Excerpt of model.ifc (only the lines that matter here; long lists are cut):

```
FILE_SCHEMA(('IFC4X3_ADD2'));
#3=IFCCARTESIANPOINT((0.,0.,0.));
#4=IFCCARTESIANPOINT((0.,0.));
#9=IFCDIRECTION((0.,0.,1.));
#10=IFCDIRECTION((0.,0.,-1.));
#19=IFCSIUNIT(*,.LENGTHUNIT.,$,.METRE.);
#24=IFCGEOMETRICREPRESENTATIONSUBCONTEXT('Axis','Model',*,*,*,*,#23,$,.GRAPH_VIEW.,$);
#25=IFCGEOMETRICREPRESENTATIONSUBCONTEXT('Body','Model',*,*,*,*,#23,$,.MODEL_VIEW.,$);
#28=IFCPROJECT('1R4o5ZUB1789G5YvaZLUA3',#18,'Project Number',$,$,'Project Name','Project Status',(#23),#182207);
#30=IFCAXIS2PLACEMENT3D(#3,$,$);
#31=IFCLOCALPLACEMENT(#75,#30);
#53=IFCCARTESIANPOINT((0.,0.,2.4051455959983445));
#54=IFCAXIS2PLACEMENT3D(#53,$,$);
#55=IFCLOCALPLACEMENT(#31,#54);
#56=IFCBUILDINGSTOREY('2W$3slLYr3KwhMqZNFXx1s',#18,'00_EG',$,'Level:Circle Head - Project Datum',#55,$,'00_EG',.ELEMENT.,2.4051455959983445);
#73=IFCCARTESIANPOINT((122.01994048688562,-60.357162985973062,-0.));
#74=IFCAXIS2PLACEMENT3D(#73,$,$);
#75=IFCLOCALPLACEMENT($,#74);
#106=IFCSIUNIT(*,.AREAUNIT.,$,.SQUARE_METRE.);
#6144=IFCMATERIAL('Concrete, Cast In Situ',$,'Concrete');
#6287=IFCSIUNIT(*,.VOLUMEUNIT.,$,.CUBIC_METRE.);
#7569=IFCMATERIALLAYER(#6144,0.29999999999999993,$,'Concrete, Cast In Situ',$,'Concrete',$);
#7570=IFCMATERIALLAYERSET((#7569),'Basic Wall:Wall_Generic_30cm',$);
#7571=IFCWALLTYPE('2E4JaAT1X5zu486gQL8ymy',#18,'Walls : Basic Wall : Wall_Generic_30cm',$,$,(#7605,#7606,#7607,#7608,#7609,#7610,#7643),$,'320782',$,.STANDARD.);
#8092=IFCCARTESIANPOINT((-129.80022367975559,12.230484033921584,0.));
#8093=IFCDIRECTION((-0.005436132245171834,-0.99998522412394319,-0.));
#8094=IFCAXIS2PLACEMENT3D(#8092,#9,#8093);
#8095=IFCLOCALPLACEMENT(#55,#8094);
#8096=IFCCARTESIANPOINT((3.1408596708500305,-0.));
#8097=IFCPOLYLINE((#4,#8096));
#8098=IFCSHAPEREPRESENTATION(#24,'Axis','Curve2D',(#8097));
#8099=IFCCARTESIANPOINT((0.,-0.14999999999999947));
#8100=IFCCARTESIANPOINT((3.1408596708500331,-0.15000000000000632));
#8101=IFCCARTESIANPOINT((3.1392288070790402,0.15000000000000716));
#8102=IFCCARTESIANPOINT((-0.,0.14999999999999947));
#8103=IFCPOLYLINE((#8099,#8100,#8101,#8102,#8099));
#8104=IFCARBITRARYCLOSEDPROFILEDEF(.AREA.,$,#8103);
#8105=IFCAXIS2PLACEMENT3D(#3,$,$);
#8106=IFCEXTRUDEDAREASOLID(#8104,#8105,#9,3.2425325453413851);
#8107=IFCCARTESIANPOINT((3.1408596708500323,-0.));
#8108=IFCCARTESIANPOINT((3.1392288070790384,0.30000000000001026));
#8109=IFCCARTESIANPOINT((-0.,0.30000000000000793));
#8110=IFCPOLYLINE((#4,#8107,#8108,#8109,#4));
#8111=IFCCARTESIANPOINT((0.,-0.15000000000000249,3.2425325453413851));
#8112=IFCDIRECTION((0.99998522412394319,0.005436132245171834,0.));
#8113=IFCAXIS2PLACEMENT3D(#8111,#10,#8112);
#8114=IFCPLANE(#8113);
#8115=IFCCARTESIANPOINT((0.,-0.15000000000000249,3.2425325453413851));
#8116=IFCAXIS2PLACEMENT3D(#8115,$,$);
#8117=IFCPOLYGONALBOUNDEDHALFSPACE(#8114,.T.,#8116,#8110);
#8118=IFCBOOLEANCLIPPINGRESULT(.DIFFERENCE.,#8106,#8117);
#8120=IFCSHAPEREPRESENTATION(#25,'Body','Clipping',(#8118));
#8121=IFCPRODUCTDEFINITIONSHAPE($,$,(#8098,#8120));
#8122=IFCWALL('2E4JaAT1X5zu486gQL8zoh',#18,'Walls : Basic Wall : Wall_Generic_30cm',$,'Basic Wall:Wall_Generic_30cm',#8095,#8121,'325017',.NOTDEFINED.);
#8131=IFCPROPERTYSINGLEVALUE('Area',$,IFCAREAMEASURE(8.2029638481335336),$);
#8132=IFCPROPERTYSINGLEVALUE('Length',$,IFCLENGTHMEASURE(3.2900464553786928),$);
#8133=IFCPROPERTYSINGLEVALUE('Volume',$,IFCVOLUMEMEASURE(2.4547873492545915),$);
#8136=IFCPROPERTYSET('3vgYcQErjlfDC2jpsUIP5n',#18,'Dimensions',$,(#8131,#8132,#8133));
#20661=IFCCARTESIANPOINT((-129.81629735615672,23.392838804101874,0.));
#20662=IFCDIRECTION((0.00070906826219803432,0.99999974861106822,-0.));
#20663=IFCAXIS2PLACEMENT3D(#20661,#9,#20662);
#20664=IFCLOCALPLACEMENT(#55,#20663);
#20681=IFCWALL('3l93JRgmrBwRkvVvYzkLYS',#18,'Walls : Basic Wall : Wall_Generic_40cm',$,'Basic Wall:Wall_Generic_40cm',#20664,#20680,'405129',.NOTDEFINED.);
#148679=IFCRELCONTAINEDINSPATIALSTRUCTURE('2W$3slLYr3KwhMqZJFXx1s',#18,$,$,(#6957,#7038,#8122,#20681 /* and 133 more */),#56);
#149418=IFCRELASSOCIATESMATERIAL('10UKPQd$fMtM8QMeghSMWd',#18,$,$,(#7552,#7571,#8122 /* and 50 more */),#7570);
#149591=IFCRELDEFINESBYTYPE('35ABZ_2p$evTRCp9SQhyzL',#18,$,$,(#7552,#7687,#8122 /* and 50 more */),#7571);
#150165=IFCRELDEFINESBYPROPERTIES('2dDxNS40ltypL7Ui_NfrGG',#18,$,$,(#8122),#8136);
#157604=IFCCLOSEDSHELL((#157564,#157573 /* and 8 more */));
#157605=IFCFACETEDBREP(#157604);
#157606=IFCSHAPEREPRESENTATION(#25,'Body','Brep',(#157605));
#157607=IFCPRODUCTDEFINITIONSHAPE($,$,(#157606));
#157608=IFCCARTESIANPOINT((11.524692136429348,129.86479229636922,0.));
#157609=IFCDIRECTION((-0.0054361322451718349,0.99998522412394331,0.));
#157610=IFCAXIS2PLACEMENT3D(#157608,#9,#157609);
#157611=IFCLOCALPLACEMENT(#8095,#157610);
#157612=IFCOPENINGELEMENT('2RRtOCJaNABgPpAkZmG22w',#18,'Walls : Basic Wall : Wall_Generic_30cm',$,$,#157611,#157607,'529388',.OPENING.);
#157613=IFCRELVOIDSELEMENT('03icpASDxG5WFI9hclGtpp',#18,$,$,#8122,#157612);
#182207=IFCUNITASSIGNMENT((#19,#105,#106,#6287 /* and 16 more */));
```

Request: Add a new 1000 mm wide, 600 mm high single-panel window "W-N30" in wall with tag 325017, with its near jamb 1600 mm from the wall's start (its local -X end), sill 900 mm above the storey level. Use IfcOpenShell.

```python
import numpy as np
import ifcopenshell
import ifcopenshell.api.feature
import ifcopenshell.api.geometry
import ifcopenshell.api.pset
import ifcopenshell.api.root
import ifcopenshell.api.spatial
import ifcopenshell.geom
import ifcopenshell.util.element
import ifcopenshell.util.placement
import ifcopenshell.util.representation
import ifcopenshell.util.shape
import ifcopenshell.util.unit

model = ifcopenshell.open("model.ifc")
unit_scale = ifcopenshell.util.unit.calculate_unit_scale(model)
area_scale = ifcopenshell.util.unit.calculate_unit_scale(model, "AREAUNIT")
volume_scale = ifcopenshell.util.unit.calculate_unit_scale(model, "VOLUMEUNIT")
settings = ifcopenshell.geom.settings()


def volume(element):
    """Net volume in cubic metres, openings subtracted."""
    shape = ifcopenshell.geom.create_shape(settings, element)
    return ifcopenshell.util.shape.get_volume(shape.geometry)


wall = model.by_guid("2E4JaAT1X5zu486gQL8zoh")
storey = ifcopenshell.util.element.get_container(wall, ifc_class="IfcBuildingStorey")
context = ifcopenshell.util.representation.get_context(model, "Model", "Body", "MODEL_VIEW")
before = volume(wall)

width, height, from_end, sill = 1, 0.6, 1.6, 0.9  # metres

# The wall runs along its own X axis, and the end named is its -X end.
wall_shape = ifcopenshell.geom.create_shape(settings, wall)
x, y, z = ifcopenshell.util.shape.get_vertices(wall_shape.geometry).T
start = x.min() + from_end
face, thickness = float(y.min()), float(y.max() - y.min())
wall_matrix = ifcopenshell.util.placement.get_local_placement(wall.ObjectPlacement)
level = ifcopenshell.util.placement.get_local_placement(storey.ObjectPlacement)[2, 3]


def in_wall(x, y):
    """Placement at x, y metres in the wall's axes, at sill height."""
    matrix = wall_matrix.copy()
    matrix[:, 3] = wall_matrix @ np.array([x / unit_scale, y / unit_scale, 0.0, 1.0])
    matrix[2, 3] = level + sill / unit_scale
    return matrix


# Opening: a box that overshoots both wall faces by 50 mm.
opening = ifcopenshell.api.root.create_entity(model, ifc_class="IfcOpeningElement", predefined_type="OPENING")
box = ifcopenshell.api.geometry.add_wall_representation(
    model, context=context, length=width, height=height, thickness=thickness + 0.1
)
ifcopenshell.api.geometry.assign_representation(model, product=opening, representation=box)
ifcopenshell.api.geometry.edit_object_placement(model, product=opening, matrix=in_wall(start, face - 0.05), is_si=False)
ifcopenshell.api.feature.add_feature(model, feature=opening, element=wall)

window = ifcopenshell.api.root.create_entity(model, ifc_class="IfcWindow", name="W-N30", predefined_type="WINDOW")
window.OverallWidth, window.OverallHeight = width / unit_scale, height / unit_scale
window.PartitioningType = "SINGLE_PANEL"
body = ifcopenshell.api.geometry.add_window_representation(
    model,
    context=context,
    overall_width=window.OverallWidth,
    overall_height=window.OverallHeight,
    partition_type="SINGLE_PANEL",
)
ifcopenshell.api.geometry.assign_representation(model, product=window, representation=body)
ifcopenshell.api.spatial.assign_container(model, products=[window], relating_structure=storey)
ifcopenshell.api.feature.add_filling(model, opening=opening, element=window)

# Centre the window in the wall's thickness.
ifcopenshell.api.geometry.edit_object_placement(model, product=window, matrix=in_wall(start, face), is_si=False)
window_shape = ifcopenshell.geom.create_shape(settings, window)
depth = ifcopenshell.util.shape.get_vertices(window_shape.geometry)[:, 1]
offset = face + thickness / 2 - (depth.min() + depth.max()) / 2
ifcopenshell.api.geometry.edit_object_placement(model, product=window, matrix=in_wall(start, offset), is_si=False)

after = volume(wall)

# Update the wall's stored quantities.
pset = model.by_id(ifcopenshell.util.element.get_pset(wall, "Dimensions", should_inherit=False)["id"])
ifcopenshell.api.pset.edit_pset(model, pset=pset, properties={
    "Area": model.create_entity("IfcAreaMeasure", after / thickness / area_scale),
    "Volume": model.create_entity("IfcVolumeMeasure", after / volume_scale),
})

print(f"wall volume {before:.3f} -> {after:.3f} m3")

model.write("model_v2.ifc")
```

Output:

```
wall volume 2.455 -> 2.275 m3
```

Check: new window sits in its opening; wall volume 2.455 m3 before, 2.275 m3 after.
